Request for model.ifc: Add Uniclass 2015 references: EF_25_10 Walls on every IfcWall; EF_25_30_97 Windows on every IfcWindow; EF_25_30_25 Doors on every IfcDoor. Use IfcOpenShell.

First a look at what the model holds.

```python
import ifcopenshell

model = ifcopenshell.open("model.ifc")
print(model.schema)
print("classifications:", [c.Name for c in model.by_type("IfcClassification")])
for ifc_class in ("IfcDoor", "IfcRoof", "IfcStair", "IfcWall", "IfcWindow"):
    print(ifc_class, len(model.by_type(ifc_class)))
```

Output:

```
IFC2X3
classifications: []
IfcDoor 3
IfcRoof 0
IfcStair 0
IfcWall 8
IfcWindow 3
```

```python
import ifcopenshell
import ifcopenshell.api.classification

model = ifcopenshell.open("model.ifc")

# IFC2X3 requires Source and Edition and has no link from the project to the system.
system = model.create_entity("IfcClassification", Source="NBS", Edition="2015", Name="Uniclass 2015")

codes = {
    "IfcWall": ("EF_25_10", "Walls"),
    "IfcWindow": ("EF_25_30_97", "Windows"),
    "IfcDoor": ("EF_25_30_25", "Doors"),
}
for ifc_class, (code, name) in codes.items():
    products = model.by_type(ifc_class)
    ifcopenshell.api.classification.add_reference(
        model, products=products, classification=system, identification=code, name=name
    )
    print(code, len(products))

model.write("model-out.ifc")
```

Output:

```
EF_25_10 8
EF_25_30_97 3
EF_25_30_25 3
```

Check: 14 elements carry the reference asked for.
